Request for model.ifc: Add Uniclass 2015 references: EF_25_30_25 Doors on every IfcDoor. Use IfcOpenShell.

First a look at what the model holds.

```python
import ifcopenshell

model = ifcopenshell.open("model.ifc")
print(model.schema)
print("classifications:", [c.Name for c in model.by_type("IfcClassification")])
for ifc_class in ("IfcDoor", "IfcRoof", "IfcStair", "IfcWall", "IfcWindow"):
    print(ifc_class, len(model.by_type(ifc_class)))
```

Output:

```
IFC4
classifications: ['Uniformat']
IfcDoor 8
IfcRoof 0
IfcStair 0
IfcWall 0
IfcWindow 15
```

```python
import ifcopenshell
import ifcopenshell.api.classification

model = ifcopenshell.open("model.ifc")

system = ifcopenshell.api.classification.add_classification(model, classification="Uniclass 2015")

codes = {
    "IfcDoor": ("EF_25_30_25", "Doors"),
}
for ifc_class, (code, name) in codes.items():
    products = model.by_type(ifc_class)
    ifcopenshell.api.classification.add_reference(
        model, products=products, classification=system, identification=code, name=name
    )
    print(code, len(products))

model.write("model_v2.ifc")
```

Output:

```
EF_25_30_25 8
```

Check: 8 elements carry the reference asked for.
